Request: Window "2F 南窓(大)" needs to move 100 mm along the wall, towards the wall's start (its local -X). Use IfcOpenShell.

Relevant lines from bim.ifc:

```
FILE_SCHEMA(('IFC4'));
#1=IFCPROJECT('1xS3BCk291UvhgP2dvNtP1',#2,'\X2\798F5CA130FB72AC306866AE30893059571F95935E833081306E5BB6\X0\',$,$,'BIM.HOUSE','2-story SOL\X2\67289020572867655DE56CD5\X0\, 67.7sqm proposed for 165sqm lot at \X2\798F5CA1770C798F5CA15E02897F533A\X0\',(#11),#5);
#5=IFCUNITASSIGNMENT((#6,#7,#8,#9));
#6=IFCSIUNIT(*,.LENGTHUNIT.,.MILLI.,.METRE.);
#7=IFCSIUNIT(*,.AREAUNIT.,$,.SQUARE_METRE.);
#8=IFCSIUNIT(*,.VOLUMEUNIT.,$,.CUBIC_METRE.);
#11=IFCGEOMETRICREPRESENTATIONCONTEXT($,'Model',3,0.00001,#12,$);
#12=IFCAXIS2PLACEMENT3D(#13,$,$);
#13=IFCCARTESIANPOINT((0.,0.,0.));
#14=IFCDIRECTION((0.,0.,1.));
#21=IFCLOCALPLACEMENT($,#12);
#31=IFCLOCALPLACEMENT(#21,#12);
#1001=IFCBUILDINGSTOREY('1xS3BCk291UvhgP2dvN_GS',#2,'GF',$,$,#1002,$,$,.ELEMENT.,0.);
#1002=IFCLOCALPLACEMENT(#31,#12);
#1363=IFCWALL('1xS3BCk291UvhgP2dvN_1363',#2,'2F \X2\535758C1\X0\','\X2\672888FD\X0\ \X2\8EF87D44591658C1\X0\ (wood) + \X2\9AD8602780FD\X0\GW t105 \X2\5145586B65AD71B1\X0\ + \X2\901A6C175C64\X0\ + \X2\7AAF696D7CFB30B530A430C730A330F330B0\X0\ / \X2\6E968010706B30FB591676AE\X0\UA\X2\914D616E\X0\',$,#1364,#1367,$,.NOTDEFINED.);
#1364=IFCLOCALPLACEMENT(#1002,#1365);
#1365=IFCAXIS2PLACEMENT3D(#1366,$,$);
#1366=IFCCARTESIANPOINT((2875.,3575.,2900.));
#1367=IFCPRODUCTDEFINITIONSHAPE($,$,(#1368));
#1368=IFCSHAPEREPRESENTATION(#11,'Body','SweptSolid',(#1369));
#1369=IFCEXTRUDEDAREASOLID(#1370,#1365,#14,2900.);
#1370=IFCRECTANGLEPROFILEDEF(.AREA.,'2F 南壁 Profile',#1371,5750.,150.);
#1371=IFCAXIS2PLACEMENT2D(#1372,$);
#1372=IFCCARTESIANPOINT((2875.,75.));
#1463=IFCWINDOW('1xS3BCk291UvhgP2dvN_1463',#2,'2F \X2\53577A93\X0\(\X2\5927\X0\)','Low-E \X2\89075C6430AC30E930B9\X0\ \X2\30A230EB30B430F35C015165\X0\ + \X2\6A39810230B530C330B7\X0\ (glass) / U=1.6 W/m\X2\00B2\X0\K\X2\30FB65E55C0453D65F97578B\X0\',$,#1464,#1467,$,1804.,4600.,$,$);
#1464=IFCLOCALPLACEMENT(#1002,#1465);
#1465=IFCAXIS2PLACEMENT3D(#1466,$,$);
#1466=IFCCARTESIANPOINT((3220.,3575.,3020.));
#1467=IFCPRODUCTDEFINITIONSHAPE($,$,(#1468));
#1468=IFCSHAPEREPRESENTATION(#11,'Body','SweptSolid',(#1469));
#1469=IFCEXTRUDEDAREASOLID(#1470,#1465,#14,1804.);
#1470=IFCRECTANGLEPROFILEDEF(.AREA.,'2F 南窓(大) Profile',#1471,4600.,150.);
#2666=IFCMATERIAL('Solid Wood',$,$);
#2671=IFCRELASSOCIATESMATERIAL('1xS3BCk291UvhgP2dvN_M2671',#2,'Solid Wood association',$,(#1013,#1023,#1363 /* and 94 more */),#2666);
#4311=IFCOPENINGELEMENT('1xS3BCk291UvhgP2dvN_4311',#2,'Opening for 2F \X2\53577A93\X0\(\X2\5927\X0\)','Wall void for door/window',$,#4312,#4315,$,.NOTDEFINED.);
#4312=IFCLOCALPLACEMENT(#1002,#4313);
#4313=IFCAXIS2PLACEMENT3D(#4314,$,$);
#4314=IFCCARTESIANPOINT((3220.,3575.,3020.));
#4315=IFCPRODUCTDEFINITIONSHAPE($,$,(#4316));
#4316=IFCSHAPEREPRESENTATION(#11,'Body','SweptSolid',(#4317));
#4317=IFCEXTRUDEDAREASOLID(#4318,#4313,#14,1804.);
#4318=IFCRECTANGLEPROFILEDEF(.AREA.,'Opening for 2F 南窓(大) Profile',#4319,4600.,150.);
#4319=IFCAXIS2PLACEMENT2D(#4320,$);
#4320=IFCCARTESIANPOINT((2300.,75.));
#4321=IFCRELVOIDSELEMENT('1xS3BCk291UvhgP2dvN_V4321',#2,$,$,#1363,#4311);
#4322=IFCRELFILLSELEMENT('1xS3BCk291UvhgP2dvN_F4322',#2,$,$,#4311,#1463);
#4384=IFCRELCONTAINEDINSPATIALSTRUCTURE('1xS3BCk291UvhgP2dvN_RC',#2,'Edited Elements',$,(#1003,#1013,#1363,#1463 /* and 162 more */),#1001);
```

```python
import ifcopenshell
import ifcopenshell.api.geometry
import ifcopenshell.util.placement

model = ifcopenshell.open("bim.ifc")

window = model.by_guid("1xS3BCk291UvhgP2dvN_1463")
opening = window.FillsVoids[0].RelatingOpeningElement
wall = opening.VoidsElements[0].RelatingBuildingElement

wall_matrix = ifcopenshell.util.placement.get_local_placement(wall.ObjectPlacement)
shift = wall_matrix[:3, 0] * -100.0
before = ifcopenshell.util.placement.get_local_placement(window.ObjectPlacement)[:3, 3].copy()

# The window is not placed relative to its opening, so move both.
for product in (opening, window):
    matrix = ifcopenshell.util.placement.get_local_placement(product.ObjectPlacement)
    matrix[:3, 3] += shift
    ifcopenshell.api.geometry.edit_object_placement(model, product=product, matrix=matrix, is_si=False)

after = ifcopenshell.util.placement.get_local_placement(window.ObjectPlacement)[:3, 3]
print("window moved by", (after - before).round(3) + 0.0)

model.write("bim-out.ifc")
```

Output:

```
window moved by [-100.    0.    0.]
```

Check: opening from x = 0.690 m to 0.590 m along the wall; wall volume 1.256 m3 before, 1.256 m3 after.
